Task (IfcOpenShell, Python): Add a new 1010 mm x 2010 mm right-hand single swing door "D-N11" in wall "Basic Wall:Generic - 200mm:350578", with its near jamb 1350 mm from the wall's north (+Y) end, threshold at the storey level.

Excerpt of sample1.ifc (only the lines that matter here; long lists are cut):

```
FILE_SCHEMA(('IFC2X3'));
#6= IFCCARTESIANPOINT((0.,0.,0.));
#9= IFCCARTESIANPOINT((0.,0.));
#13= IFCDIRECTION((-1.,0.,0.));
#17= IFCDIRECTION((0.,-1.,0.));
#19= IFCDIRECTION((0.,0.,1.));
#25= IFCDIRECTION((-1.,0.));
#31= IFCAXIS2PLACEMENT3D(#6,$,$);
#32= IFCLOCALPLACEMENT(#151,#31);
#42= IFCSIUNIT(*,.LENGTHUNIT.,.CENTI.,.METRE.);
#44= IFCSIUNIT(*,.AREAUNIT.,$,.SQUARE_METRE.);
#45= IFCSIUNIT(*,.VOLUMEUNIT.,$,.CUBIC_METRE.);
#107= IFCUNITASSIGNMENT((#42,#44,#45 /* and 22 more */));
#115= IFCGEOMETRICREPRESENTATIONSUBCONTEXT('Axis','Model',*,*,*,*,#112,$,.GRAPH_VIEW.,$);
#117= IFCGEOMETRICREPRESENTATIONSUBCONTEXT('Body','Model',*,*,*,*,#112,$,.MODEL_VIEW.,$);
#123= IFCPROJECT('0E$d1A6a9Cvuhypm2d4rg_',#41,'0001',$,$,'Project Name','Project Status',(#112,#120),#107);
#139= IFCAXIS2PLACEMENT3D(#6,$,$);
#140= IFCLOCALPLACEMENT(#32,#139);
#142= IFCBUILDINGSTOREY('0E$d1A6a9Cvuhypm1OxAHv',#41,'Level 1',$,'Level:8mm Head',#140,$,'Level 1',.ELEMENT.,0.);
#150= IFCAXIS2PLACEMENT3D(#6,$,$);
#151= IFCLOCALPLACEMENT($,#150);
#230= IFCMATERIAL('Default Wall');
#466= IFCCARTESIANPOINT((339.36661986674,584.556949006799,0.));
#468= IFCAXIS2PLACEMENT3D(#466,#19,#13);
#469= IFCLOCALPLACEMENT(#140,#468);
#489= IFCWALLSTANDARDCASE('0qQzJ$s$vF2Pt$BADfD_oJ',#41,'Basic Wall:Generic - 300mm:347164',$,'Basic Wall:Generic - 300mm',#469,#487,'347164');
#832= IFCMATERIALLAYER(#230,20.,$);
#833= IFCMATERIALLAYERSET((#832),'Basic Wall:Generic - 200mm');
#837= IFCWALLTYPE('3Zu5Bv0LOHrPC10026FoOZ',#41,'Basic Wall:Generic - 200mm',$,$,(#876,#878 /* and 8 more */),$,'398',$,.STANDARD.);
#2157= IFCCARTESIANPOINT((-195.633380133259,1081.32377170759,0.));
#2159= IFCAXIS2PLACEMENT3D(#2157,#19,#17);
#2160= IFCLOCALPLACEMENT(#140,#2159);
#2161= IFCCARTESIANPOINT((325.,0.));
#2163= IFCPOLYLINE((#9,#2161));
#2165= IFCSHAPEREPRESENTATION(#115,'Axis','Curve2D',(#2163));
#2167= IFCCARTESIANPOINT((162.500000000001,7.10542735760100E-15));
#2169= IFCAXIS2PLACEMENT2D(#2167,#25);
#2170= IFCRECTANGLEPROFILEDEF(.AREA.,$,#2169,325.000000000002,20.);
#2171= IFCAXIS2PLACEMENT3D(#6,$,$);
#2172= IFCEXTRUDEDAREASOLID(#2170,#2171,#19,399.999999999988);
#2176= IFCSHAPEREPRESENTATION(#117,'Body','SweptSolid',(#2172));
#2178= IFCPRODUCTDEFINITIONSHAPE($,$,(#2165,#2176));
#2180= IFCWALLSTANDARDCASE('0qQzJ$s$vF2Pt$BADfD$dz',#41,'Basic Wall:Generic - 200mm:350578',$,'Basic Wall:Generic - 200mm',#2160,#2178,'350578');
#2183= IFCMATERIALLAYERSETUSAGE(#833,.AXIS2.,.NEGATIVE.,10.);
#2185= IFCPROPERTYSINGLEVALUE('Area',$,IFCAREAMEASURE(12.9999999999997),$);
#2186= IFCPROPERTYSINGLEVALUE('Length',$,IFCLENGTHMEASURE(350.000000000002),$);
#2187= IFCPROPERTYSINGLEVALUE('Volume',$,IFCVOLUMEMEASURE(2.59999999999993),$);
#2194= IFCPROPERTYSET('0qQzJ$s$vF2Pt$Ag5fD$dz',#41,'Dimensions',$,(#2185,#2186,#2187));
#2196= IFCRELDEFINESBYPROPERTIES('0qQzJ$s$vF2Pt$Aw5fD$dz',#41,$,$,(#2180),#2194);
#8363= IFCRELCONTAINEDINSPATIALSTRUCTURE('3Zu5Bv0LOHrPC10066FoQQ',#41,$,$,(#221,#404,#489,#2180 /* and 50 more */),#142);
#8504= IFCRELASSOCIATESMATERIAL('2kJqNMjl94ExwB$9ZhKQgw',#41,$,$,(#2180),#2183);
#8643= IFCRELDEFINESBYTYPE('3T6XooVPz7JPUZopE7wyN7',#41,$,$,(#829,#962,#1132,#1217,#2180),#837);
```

```python
import numpy as np
import ifcopenshell
import ifcopenshell.api.feature
import ifcopenshell.api.geometry
import ifcopenshell.api.pset
import ifcopenshell.api.root
import ifcopenshell.api.spatial
import ifcopenshell.api.type
import ifcopenshell.geom
import ifcopenshell.util.element
import ifcopenshell.util.placement
import ifcopenshell.util.representation
import ifcopenshell.util.shape
import ifcopenshell.util.unit

model = ifcopenshell.open("sample1.ifc")
unit_scale = ifcopenshell.util.unit.calculate_unit_scale(model)
area_scale = ifcopenshell.util.unit.calculate_unit_scale(model, "AREAUNIT")
volume_scale = ifcopenshell.util.unit.calculate_unit_scale(model, "VOLUMEUNIT")
settings = ifcopenshell.geom.settings()


def volume(element):
    """Net volume in cubic metres, openings subtracted."""
    shape = ifcopenshell.geom.create_shape(settings, element)
    return ifcopenshell.util.shape.get_volume(shape.geometry)


wall = model.by_guid("0qQzJ$s$vF2Pt$BADfD$dz")
storey = ifcopenshell.util.element.get_container(wall, ifc_class="IfcBuildingStorey")
context = ifcopenshell.util.representation.get_context(model, "Model", "Body", "MODEL_VIEW")
before = volume(wall)

width, height, from_end, sill = 1.01, 2.01, 1.35, 0.0  # metres

# The wall runs along its own X axis, and the end named is its -X end.
wall_shape = ifcopenshell.geom.create_shape(settings, wall)
x, y, z = ifcopenshell.util.shape.get_vertices(wall_shape.geometry).T
start = x.min() + from_end
face, thickness = float(y.min()), float(y.max() - y.min())
wall_matrix = ifcopenshell.util.placement.get_local_placement(wall.ObjectPlacement)
level = ifcopenshell.util.placement.get_local_placement(storey.ObjectPlacement)[2, 3]


def in_wall(x, y):
    """Placement at x, y metres in the wall's axes, at sill height."""
    matrix = wall_matrix.copy()
    matrix[:, 3] = wall_matrix @ np.array([x / unit_scale, y / unit_scale, 0.0, 1.0])
    matrix[2, 3] = level + sill / unit_scale
    return matrix


# Opening: a box that overshoots both wall faces by 50 mm.
opening = ifcopenshell.api.root.create_entity(model, ifc_class="IfcOpeningElement")
box = ifcopenshell.api.geometry.add_wall_representation(
    model, context=context, length=width, height=height, thickness=thickness + 0.1
)
ifcopenshell.api.geometry.assign_representation(model, product=opening, representation=box)
ifcopenshell.api.geometry.edit_object_placement(model, product=opening, matrix=in_wall(start, face - 0.05), is_si=False)
ifcopenshell.api.feature.add_feature(model, feature=opening, element=wall)

door = ifcopenshell.api.root.create_entity(model, ifc_class="IfcDoor", name="D-N11")
door.OverallWidth, door.OverallHeight = width / unit_scale, height / unit_scale
body = ifcopenshell.api.geometry.add_door_representation(
    model,
    context=context,
    overall_width=door.OverallWidth,
    overall_height=door.OverallHeight,
    operation_type="SINGLE_SWING_RIGHT",
    lining_properties={"LiningDepth": thickness / unit_scale, "ThresholdDepth": thickness / unit_scale},
)
ifcopenshell.api.geometry.assign_representation(model, product=door, representation=body)
ifcopenshell.api.spatial.assign_container(model, products=[door], relating_structure=storey)
fills = ifcopenshell.api.feature.add_filling(model, opening=opening, element=door)
fills.OwnerHistory = door.OwnerHistory  # required in IFC2X3

# IFC2X3 keeps the operation on the door style.
style = ifcopenshell.api.root.create_entity(model, ifc_class="IfcDoorStyle", name="D-N11")
style.OperationType, style.ConstructionType = "SINGLE_SWING_RIGHT", "NOTDEFINED"
style.ParameterTakesPrecedence = style.Sizeable = False
ifcopenshell.api.type.assign_type(model, related_objects=[door], relating_type=style)

# The lining spans the wall, so the door starts at the wall face.
ifcopenshell.api.geometry.edit_object_placement(model, product=door, matrix=in_wall(start, face), is_si=False)

after = volume(wall)

# Update the wall's stored quantities.
pset = model.by_id(ifcopenshell.util.element.get_pset(wall, "Dimensions", should_inherit=False)["id"])
ifcopenshell.api.pset.edit_pset(model, pset=pset, properties={
    "Area": model.create_entity("IfcAreaMeasure", after / thickness / area_scale),
    "Volume": model.create_entity("IfcVolumeMeasure", after / volume_scale),
})

print(f"wall volume {before:.3f} -> {after:.3f} m3")

model.write("sample1_edited.ifc")
```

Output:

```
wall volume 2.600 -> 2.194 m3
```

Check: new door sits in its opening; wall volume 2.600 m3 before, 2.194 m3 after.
